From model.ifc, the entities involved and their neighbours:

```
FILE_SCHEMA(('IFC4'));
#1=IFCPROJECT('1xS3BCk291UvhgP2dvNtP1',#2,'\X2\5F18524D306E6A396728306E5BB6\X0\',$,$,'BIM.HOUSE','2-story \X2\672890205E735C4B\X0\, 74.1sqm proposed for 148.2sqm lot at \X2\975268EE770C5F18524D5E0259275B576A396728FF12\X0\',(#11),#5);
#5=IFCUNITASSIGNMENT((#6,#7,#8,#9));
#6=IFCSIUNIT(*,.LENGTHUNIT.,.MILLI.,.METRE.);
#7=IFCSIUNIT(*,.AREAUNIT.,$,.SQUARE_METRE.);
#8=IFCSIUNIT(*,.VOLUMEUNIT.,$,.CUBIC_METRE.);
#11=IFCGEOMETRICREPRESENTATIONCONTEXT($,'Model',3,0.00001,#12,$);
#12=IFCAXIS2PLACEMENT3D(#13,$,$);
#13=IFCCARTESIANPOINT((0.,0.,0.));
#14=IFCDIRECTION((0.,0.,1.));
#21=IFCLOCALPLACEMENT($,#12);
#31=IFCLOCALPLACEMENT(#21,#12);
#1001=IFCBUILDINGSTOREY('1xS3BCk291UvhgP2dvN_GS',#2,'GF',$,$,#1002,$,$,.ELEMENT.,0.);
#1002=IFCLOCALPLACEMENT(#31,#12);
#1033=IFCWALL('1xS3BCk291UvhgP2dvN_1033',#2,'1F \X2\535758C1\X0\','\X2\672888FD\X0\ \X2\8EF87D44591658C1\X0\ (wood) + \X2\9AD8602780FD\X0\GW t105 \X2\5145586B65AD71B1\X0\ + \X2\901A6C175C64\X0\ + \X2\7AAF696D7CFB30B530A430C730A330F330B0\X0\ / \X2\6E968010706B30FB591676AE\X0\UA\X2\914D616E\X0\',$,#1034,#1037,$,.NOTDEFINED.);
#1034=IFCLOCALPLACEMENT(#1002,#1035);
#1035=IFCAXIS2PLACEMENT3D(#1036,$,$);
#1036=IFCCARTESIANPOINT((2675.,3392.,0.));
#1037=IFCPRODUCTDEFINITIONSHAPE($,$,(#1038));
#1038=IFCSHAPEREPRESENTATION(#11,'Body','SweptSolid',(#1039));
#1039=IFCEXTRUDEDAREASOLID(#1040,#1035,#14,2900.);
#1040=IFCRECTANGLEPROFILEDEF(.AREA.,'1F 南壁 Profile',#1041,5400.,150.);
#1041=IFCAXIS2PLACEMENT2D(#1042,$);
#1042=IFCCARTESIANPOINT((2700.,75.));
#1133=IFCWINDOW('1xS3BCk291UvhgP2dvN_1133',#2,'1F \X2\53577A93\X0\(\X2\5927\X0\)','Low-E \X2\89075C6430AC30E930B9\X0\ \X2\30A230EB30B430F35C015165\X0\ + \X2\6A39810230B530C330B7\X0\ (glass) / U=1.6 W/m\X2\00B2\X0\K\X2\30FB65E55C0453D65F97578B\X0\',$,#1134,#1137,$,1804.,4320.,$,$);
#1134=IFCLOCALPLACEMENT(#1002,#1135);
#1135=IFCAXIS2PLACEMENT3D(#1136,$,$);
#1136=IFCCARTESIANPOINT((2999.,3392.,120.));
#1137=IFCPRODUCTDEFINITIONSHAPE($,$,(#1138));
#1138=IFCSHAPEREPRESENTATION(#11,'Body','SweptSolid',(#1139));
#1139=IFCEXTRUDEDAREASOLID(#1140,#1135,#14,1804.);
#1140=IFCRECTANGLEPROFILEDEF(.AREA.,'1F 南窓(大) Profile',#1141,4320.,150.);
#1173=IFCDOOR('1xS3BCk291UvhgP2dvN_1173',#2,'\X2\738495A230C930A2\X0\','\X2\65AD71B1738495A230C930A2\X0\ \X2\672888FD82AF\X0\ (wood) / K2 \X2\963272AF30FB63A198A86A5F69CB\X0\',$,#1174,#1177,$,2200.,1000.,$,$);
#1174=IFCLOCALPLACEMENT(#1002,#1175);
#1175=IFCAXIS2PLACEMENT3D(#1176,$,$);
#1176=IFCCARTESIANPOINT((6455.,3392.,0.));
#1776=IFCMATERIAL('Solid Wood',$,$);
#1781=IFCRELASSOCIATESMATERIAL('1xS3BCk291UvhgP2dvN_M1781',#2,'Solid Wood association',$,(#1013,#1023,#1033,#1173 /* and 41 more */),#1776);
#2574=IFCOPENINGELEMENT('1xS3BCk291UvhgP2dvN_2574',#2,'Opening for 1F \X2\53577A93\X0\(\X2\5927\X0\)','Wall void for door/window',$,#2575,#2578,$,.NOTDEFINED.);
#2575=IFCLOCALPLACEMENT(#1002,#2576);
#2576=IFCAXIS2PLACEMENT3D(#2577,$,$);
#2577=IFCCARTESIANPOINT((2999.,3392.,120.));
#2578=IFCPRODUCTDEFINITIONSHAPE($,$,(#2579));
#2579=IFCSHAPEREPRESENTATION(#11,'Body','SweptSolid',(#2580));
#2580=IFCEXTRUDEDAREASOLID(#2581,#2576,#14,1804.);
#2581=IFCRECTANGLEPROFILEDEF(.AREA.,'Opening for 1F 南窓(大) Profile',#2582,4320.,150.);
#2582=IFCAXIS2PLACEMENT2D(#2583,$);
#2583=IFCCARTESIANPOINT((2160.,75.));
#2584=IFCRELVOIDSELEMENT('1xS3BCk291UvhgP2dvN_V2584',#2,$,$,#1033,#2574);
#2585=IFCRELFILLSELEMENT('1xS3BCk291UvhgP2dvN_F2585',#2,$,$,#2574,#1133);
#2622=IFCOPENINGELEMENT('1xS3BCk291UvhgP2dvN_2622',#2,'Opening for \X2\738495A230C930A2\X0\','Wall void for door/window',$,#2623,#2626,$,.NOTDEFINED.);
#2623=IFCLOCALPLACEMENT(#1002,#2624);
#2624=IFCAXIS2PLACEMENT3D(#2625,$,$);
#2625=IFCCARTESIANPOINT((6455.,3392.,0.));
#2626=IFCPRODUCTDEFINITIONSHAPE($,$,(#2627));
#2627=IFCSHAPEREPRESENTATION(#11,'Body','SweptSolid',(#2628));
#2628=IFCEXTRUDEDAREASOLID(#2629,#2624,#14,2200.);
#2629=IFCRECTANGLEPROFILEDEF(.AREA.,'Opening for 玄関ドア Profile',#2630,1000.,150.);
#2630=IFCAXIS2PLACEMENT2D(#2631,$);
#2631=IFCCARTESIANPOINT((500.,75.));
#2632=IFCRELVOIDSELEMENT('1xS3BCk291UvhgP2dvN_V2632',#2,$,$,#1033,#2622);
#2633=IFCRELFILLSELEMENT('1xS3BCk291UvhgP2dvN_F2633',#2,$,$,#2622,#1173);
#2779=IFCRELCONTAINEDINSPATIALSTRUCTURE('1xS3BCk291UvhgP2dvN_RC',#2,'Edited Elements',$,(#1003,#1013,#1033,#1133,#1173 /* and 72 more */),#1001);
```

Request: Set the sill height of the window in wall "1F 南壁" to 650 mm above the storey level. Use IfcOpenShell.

```python
import numpy as np
import ifcopenshell
import ifcopenshell.api.geometry
import ifcopenshell.geom
import ifcopenshell.util.element
import ifcopenshell.util.placement
import ifcopenshell.util.shape
import ifcopenshell.util.unit

model = ifcopenshell.open("model.ifc")
unit_scale = ifcopenshell.util.unit.calculate_unit_scale(model)

window = model.by_guid("1xS3BCk291UvhgP2dvN_1133")
opening = window.FillsVoids[0].RelatingOpeningElement
storey = ifcopenshell.util.element.get_container(window, ifc_class="IfcBuildingStorey")
level = ifcopenshell.util.placement.get_local_placement(storey.ObjectPlacement)[2, 3]

# The opening's origin need not be at the sill, so measure its lowest point.
shape = ifcopenshell.geom.create_shape(ifcopenshell.geom.settings(), opening)
bottom = ifcopenshell.util.shape.get_shape_bottom_elevation(shape, shape.geometry) / unit_scale
dz = level + 650.0 - bottom

shift = np.array([0.0, 0.0, dz])
# The window is not placed relative to its opening, so move both.
for product in (opening, window):
    matrix = ifcopenshell.util.placement.get_local_placement(product.ObjectPlacement)
    matrix[:3, 3] += shift
    ifcopenshell.api.geometry.edit_object_placement(model, product=product, matrix=matrix, is_si=False)

print(f"moved by {dz * unit_scale:+.3f} m")

model.write("model_v2.ifc")
```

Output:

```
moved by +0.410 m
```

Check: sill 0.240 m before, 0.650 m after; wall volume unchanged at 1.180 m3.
